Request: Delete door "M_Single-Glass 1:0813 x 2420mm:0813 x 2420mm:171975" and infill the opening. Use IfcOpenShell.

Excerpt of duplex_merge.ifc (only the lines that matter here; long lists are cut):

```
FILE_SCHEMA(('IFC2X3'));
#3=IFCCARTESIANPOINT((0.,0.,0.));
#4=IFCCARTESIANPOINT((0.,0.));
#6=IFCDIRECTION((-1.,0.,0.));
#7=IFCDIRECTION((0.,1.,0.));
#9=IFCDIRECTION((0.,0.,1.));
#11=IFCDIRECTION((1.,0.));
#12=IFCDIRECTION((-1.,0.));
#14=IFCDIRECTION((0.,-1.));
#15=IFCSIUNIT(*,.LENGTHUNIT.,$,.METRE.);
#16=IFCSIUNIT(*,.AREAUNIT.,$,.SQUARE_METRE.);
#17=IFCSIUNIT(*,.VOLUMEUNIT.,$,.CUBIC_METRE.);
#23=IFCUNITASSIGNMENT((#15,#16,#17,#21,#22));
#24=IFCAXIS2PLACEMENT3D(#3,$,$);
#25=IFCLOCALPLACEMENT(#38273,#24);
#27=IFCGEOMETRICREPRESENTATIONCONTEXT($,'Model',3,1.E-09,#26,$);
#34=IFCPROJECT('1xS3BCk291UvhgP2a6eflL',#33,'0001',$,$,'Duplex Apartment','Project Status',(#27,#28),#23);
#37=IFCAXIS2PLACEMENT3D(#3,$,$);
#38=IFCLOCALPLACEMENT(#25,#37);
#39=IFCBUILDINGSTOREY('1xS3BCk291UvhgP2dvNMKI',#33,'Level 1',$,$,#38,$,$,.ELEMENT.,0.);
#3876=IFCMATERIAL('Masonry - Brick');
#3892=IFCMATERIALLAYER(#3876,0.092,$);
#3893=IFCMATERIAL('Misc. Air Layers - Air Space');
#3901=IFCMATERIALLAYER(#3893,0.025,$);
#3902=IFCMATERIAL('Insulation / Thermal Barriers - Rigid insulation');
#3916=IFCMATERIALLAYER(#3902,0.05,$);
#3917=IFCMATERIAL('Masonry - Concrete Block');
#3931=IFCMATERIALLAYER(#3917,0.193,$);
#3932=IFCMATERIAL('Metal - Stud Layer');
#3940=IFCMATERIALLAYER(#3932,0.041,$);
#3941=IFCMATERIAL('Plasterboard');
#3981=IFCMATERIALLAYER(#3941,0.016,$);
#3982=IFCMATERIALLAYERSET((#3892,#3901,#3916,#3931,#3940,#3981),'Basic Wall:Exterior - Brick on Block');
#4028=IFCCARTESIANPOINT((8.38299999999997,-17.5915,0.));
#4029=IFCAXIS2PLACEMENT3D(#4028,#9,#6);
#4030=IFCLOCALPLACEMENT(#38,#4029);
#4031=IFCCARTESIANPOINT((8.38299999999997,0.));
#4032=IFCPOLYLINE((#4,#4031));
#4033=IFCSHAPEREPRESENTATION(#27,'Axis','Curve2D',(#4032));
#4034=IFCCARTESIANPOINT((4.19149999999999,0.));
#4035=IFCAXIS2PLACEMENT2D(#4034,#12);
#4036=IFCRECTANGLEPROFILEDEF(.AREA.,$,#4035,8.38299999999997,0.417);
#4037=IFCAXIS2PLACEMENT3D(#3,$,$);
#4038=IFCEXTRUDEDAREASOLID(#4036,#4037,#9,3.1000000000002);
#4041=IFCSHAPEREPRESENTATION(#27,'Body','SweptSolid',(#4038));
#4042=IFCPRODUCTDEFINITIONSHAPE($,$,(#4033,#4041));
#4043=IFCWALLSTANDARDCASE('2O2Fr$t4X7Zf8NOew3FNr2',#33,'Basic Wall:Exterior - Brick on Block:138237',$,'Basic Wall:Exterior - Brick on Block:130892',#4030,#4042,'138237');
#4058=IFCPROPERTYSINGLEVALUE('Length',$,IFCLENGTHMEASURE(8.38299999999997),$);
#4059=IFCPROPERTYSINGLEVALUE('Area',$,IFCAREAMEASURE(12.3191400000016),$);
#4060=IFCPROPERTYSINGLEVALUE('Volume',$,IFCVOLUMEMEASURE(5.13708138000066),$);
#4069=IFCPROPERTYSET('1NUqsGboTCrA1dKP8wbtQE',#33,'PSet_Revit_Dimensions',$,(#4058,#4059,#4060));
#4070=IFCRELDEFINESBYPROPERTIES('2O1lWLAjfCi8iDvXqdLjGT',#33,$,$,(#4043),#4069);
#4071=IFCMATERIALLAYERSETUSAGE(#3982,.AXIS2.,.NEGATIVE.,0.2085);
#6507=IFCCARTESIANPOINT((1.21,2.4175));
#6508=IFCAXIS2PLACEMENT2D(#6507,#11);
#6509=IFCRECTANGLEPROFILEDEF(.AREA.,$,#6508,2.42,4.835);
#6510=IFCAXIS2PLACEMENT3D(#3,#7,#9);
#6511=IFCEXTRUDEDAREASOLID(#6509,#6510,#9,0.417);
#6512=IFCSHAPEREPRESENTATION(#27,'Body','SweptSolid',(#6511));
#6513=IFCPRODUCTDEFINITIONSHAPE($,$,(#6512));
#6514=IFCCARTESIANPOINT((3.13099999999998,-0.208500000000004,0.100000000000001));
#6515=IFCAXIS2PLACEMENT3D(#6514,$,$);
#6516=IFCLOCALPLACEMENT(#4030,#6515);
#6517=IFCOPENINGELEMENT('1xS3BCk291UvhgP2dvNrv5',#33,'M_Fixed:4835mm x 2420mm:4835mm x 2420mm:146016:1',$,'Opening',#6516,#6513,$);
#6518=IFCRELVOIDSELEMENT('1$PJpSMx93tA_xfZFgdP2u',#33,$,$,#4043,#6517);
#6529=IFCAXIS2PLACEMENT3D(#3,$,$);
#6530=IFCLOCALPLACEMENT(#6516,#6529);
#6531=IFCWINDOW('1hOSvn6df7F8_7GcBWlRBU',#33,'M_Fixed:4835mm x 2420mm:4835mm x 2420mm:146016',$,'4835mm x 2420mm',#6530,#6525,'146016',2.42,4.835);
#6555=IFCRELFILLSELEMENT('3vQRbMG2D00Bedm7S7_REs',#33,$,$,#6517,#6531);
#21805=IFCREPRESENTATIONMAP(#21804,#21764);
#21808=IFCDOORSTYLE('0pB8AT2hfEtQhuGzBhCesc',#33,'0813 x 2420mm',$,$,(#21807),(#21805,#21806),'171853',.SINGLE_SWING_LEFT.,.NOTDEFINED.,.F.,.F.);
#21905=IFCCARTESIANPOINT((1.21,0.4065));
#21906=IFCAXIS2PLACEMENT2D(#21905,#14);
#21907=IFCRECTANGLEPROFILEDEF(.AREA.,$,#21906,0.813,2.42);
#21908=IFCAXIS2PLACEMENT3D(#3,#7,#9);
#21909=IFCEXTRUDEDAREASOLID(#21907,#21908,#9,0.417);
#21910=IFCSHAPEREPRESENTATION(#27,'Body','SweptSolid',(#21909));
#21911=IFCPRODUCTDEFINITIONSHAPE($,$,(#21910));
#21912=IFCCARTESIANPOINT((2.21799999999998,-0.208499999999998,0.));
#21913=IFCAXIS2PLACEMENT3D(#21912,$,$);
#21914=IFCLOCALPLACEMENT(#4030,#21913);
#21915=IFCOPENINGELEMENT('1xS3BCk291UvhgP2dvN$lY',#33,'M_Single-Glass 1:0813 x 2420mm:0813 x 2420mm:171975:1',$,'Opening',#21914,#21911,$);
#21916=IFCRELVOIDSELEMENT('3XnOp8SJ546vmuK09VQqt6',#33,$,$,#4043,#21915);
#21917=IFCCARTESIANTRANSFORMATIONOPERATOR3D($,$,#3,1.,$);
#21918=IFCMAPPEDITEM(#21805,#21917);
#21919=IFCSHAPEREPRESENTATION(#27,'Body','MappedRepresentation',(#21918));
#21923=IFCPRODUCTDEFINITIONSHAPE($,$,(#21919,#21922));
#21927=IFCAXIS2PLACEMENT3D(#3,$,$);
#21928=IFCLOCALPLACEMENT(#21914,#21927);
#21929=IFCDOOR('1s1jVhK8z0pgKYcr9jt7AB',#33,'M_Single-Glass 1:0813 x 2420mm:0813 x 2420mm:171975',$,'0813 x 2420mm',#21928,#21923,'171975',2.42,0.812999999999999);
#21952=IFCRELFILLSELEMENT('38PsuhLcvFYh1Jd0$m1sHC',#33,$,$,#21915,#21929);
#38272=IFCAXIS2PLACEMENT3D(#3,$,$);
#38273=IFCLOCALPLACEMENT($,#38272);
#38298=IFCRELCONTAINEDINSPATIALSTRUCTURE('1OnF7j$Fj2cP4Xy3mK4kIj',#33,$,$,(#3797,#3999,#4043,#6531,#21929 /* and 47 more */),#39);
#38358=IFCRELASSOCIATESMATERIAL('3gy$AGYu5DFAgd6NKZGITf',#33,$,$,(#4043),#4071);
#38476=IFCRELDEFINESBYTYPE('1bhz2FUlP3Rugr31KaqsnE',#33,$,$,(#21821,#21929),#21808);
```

```python
import ifcopenshell
import ifcopenshell.api.feature
import ifcopenshell.api.pset
import ifcopenshell.api.root
import ifcopenshell.geom
import ifcopenshell.util.element
import ifcopenshell.util.shape
import ifcopenshell.util.unit

model = ifcopenshell.open("duplex_merge.ifc")
area_scale = ifcopenshell.util.unit.calculate_unit_scale(model, "AREAUNIT")
volume_scale = ifcopenshell.util.unit.calculate_unit_scale(model, "VOLUMEUNIT")
settings = ifcopenshell.geom.settings()


def volume(element):
    """Net volume in cubic metres, openings subtracted."""
    shape = ifcopenshell.geom.create_shape(settings, element)
    return ifcopenshell.util.shape.get_volume(shape.geometry)


door = model.by_guid("1s1jVhK8z0pgKYcr9jt7AB")
opening = door.FillsVoids[0].RelatingOpeningElement
wall = opening.VoidsElements[0].RelatingBuildingElement
before = volume(wall)

ifcopenshell.api.root.remove_product(model, product=door)
ifcopenshell.api.feature.remove_feature(model, feature=opening)

after = volume(wall)
thickness = 0.417  # wall thickness in metres

# Update the wall's stored quantities.
pset = model.by_id(ifcopenshell.util.element.get_pset(wall, "PSet_Revit_Dimensions", should_inherit=False)["id"])
ifcopenshell.api.pset.edit_pset(model, pset=pset, properties={
    "Area": model.create_entity("IfcAreaMeasure", after / thickness / area_scale),
    "Volume": model.create_entity("IfcVolumeMeasure", after / volume_scale),
})

print(f"wall volume {before:.3f} -> {after:.3f} m3")

model.write("duplex_merge_v2.ifc")
```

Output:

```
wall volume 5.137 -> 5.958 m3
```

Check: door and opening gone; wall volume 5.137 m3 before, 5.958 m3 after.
